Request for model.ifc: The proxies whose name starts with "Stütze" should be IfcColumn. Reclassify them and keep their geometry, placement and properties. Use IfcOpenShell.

First a look at what the model holds.

```python
import re

import ifcopenshell

model = ifcopenshell.open("model.ifc")
print(model.schema)
seen = {}
for e in model.by_type("IfcBuildingElementProxy"):
    name = re.sub(r":\d+(:\d+)?$", "", e.Name or "")  # drop the element id that some exporters append
    seen[name] = seen.get(name, 0) + 1
for name, count in sorted(seen.items()):
    print(count, "x", name)
```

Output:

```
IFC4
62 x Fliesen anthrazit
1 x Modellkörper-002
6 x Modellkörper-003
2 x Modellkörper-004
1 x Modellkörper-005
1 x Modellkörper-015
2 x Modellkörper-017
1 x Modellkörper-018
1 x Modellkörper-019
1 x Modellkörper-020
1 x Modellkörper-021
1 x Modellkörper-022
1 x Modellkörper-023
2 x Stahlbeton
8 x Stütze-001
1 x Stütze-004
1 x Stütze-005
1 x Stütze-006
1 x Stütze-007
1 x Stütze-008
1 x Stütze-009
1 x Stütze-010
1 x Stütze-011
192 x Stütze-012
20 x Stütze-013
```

```python
import ifcopenshell
import ifcopenshell.api.root

model = ifcopenshell.open("model.ifc")

proxies = [e.id() for e in model.by_type("IfcBuildingElementProxy") if (e.Name or "").startswith("Stütze")]
for step_id in proxies:
    proxy = model.by_id(step_id)
    # Reclassifying a typed element also reclassifies its type and the type's other occurrences.
    if proxy.is_a("IfcBuildingElementProxy"):
        ifcopenshell.api.root.reassign_class(model, product=proxy, ifc_class="IfcColumn")

print(sum(model.by_id(i).is_a("IfcColumn") for i in proxies), "reclassified")

model.write("model_updated.ifc")
```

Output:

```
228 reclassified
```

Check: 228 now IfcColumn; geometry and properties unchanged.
